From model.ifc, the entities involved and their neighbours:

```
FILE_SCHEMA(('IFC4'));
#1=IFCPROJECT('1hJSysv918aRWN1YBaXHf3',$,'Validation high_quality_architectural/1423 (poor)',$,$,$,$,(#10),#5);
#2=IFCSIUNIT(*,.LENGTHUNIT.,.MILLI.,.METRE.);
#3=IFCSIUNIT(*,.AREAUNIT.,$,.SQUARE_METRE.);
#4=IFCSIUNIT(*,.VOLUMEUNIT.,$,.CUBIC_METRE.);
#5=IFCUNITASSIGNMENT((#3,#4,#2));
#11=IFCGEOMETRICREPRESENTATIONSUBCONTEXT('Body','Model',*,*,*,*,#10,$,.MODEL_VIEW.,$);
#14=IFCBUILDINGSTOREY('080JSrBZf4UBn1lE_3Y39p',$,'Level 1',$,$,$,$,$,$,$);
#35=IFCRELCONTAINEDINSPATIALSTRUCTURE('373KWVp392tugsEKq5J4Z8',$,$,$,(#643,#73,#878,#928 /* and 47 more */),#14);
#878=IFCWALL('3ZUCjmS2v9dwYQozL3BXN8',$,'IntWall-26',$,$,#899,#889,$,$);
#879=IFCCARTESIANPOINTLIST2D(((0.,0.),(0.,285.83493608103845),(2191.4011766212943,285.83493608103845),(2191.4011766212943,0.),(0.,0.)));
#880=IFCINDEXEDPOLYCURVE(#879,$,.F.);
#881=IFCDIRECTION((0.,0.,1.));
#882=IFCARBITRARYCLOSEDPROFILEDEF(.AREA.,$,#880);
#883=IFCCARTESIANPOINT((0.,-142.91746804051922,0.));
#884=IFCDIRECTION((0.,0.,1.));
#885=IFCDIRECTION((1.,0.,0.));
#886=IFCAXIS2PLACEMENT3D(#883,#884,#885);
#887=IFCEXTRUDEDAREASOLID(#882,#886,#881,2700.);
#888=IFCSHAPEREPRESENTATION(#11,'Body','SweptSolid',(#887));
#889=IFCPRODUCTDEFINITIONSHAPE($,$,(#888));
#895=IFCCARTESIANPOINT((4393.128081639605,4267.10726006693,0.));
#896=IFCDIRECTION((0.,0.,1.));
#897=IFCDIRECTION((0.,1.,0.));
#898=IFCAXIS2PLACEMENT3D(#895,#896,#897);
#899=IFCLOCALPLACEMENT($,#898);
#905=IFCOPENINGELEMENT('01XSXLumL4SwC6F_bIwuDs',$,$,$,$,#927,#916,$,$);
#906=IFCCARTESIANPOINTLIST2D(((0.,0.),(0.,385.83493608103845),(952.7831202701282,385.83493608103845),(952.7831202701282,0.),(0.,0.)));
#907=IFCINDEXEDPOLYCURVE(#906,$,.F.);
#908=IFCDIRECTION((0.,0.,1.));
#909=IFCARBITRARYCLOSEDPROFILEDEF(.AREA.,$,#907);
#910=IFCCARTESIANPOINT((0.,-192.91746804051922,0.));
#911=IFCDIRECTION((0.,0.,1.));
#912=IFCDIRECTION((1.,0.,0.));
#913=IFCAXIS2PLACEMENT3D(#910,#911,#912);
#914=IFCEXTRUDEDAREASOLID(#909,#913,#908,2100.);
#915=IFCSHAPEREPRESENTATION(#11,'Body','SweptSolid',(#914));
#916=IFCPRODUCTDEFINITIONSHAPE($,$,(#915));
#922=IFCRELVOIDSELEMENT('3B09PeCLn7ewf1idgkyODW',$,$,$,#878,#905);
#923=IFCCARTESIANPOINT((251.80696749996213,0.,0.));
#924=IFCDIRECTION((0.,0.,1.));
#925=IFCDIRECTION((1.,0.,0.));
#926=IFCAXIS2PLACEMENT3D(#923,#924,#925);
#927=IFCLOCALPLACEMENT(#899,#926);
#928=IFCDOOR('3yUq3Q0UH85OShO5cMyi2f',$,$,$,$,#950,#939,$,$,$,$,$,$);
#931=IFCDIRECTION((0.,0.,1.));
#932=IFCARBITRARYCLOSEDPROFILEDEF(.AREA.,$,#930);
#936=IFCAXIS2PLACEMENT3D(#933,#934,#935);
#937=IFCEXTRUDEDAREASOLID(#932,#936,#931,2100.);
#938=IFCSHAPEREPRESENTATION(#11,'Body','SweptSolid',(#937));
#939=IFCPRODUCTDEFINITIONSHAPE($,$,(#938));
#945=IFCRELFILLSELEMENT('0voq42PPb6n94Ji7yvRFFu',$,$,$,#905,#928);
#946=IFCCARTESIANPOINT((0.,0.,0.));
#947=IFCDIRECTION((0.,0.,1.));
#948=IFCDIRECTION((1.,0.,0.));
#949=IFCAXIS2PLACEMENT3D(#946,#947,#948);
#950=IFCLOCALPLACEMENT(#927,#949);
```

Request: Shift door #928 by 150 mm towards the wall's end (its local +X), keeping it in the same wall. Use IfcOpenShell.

```python
import ifcopenshell
import ifcopenshell.api.geometry
import ifcopenshell.util.placement
import ifcopenshell.util.unit

model = ifcopenshell.open("model.ifc")
unit_scale = ifcopenshell.util.unit.calculate_unit_scale(model)

door = model.by_guid("3yUq3Q0UH85OShO5cMyi2f")
opening = door.FillsVoids[0].RelatingOpeningElement
wall = opening.VoidsElements[0].RelatingBuildingElement

wall_matrix = ifcopenshell.util.placement.get_local_placement(wall.ObjectPlacement)
shift = wall_matrix[:3, 0] * 0.15 / unit_scale
before = ifcopenshell.util.placement.get_local_placement(door.ObjectPlacement)[:3, 3].copy()

# The door is placed relative to its opening, so it follows when the opening moves.
matrix = ifcopenshell.util.placement.get_local_placement(opening.ObjectPlacement)
matrix[:3, 3] += shift
ifcopenshell.api.geometry.edit_object_placement(
    model, product=opening, matrix=matrix, is_si=False, should_transform_children=True
)

after = ifcopenshell.util.placement.get_local_placement(door.ObjectPlacement)[:3, 3]
print("door moved by", (after - before).round(3) + 0.0)

model.write("model_rev.ifc")
```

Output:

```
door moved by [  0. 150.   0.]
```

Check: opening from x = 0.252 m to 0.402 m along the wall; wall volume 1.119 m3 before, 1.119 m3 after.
